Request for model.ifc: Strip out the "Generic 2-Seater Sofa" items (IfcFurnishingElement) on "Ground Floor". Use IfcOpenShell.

First a look at what the model holds.

```python
import ifcopenshell
import ifcopenshell.util.element

model = ifcopenshell.open("model.ifc")
print(model.schema)
storey = next(s for s in model.by_type("IfcBuildingStorey") if s.Name == "Ground Floor")
furniture = [e for e in ifcopenshell.util.element.get_decomposition(storey) if e.is_a("IfcFurnishingElement")]
seen = {}
for e in furniture:
    element_type = ifcopenshell.util.element.get_type(e)
    name = element_type.Name if element_type not in (None, e) else None
    seen[name] = seen.get(name, 0) + 1
for name, count in sorted(seen.items(), key=str):
    print(count, "x", name)
```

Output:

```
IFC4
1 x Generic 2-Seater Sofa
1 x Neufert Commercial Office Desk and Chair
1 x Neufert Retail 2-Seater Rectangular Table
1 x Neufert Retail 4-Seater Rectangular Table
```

```python
import ifcopenshell
import ifcopenshell.api.root
import ifcopenshell.util.element

model = ifcopenshell.open("model.ifc")

storey = next(s for s in model.by_type("IfcBuildingStorey") if s.Name == "Ground Floor")
furniture = [e for e in ifcopenshell.util.element.get_decomposition(storey) if e.is_a("IfcFurnishingElement")]
targets = [e for e in furniture if (t := ifcopenshell.util.element.get_type(e)) not in (None, e) and t.Name == "Generic 2-Seater Sofa"]

for e in targets:
    ifcopenshell.api.root.remove_product(model, product=e)
print(len(targets), "removed")

model.write("model_edited.ifc")
```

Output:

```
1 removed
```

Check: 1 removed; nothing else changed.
